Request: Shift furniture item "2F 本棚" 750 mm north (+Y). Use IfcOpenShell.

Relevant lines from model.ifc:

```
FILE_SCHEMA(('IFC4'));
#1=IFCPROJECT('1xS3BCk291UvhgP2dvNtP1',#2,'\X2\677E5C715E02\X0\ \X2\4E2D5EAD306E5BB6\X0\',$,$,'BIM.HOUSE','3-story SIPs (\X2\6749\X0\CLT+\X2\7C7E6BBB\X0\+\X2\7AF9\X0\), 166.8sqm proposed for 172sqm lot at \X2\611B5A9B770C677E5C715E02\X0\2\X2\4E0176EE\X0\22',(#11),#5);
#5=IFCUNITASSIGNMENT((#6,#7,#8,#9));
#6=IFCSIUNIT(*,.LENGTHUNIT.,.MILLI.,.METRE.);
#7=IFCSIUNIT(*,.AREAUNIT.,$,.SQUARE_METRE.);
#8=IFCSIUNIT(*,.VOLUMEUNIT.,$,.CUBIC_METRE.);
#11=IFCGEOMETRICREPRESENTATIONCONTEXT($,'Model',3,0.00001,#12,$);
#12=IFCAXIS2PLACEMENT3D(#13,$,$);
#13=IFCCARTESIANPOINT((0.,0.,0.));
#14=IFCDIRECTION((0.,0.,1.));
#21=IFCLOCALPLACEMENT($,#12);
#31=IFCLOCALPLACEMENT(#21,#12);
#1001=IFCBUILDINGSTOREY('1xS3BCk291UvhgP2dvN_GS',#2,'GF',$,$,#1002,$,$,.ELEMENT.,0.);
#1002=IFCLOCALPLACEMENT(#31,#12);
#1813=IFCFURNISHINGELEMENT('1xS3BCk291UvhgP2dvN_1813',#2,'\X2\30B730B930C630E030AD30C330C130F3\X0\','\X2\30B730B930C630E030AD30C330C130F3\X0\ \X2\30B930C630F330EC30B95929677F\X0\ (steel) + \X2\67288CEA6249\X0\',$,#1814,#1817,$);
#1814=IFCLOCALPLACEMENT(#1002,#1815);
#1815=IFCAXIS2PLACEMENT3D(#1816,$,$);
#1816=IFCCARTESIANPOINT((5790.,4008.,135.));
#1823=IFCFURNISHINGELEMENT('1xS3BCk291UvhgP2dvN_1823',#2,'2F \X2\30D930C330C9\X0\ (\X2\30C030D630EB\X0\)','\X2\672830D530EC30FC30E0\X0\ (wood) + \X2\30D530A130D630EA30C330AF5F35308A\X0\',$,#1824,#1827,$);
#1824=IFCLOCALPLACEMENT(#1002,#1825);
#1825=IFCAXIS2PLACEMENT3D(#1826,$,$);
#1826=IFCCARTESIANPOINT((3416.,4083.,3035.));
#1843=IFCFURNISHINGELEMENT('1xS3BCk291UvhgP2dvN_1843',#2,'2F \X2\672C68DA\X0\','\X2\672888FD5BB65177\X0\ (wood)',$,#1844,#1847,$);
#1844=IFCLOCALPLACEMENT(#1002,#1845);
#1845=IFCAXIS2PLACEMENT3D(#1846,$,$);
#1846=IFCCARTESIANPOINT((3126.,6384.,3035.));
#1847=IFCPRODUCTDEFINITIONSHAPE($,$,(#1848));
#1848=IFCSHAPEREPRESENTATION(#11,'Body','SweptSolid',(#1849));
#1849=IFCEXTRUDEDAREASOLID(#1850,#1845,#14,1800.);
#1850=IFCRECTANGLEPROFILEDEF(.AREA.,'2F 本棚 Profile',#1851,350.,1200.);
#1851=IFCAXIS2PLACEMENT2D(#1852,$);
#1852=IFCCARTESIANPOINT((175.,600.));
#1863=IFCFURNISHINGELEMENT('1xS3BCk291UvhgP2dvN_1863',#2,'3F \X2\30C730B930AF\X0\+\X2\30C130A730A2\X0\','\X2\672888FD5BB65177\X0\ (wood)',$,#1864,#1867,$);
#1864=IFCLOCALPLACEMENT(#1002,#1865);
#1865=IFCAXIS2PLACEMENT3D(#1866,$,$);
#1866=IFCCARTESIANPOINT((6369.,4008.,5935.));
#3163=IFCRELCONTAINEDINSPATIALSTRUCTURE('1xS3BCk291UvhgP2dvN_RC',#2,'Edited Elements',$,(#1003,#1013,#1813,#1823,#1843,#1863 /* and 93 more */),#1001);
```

```python
import ifcopenshell
import ifcopenshell.api.geometry
import ifcopenshell.util.placement
import ifcopenshell.util.unit

model = ifcopenshell.open("model.ifc")
unit_scale = ifcopenshell.util.unit.calculate_unit_scale(model)

item = model.by_guid("1xS3BCk291UvhgP2dvN_1843")
matrix = ifcopenshell.util.placement.get_local_placement(item.ObjectPlacement)
matrix[1, 3] += 0.75 / unit_scale
ifcopenshell.api.geometry.edit_object_placement(model, product=item, matrix=matrix, is_si=False)

print(ifcopenshell.util.placement.get_local_placement(item.ObjectPlacement).round(3) + 0.0)

model.write("model_edited.ifc")
```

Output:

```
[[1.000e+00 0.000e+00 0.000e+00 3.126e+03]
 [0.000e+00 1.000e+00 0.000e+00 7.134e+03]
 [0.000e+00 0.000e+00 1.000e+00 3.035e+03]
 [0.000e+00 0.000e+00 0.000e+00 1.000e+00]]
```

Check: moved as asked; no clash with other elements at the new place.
